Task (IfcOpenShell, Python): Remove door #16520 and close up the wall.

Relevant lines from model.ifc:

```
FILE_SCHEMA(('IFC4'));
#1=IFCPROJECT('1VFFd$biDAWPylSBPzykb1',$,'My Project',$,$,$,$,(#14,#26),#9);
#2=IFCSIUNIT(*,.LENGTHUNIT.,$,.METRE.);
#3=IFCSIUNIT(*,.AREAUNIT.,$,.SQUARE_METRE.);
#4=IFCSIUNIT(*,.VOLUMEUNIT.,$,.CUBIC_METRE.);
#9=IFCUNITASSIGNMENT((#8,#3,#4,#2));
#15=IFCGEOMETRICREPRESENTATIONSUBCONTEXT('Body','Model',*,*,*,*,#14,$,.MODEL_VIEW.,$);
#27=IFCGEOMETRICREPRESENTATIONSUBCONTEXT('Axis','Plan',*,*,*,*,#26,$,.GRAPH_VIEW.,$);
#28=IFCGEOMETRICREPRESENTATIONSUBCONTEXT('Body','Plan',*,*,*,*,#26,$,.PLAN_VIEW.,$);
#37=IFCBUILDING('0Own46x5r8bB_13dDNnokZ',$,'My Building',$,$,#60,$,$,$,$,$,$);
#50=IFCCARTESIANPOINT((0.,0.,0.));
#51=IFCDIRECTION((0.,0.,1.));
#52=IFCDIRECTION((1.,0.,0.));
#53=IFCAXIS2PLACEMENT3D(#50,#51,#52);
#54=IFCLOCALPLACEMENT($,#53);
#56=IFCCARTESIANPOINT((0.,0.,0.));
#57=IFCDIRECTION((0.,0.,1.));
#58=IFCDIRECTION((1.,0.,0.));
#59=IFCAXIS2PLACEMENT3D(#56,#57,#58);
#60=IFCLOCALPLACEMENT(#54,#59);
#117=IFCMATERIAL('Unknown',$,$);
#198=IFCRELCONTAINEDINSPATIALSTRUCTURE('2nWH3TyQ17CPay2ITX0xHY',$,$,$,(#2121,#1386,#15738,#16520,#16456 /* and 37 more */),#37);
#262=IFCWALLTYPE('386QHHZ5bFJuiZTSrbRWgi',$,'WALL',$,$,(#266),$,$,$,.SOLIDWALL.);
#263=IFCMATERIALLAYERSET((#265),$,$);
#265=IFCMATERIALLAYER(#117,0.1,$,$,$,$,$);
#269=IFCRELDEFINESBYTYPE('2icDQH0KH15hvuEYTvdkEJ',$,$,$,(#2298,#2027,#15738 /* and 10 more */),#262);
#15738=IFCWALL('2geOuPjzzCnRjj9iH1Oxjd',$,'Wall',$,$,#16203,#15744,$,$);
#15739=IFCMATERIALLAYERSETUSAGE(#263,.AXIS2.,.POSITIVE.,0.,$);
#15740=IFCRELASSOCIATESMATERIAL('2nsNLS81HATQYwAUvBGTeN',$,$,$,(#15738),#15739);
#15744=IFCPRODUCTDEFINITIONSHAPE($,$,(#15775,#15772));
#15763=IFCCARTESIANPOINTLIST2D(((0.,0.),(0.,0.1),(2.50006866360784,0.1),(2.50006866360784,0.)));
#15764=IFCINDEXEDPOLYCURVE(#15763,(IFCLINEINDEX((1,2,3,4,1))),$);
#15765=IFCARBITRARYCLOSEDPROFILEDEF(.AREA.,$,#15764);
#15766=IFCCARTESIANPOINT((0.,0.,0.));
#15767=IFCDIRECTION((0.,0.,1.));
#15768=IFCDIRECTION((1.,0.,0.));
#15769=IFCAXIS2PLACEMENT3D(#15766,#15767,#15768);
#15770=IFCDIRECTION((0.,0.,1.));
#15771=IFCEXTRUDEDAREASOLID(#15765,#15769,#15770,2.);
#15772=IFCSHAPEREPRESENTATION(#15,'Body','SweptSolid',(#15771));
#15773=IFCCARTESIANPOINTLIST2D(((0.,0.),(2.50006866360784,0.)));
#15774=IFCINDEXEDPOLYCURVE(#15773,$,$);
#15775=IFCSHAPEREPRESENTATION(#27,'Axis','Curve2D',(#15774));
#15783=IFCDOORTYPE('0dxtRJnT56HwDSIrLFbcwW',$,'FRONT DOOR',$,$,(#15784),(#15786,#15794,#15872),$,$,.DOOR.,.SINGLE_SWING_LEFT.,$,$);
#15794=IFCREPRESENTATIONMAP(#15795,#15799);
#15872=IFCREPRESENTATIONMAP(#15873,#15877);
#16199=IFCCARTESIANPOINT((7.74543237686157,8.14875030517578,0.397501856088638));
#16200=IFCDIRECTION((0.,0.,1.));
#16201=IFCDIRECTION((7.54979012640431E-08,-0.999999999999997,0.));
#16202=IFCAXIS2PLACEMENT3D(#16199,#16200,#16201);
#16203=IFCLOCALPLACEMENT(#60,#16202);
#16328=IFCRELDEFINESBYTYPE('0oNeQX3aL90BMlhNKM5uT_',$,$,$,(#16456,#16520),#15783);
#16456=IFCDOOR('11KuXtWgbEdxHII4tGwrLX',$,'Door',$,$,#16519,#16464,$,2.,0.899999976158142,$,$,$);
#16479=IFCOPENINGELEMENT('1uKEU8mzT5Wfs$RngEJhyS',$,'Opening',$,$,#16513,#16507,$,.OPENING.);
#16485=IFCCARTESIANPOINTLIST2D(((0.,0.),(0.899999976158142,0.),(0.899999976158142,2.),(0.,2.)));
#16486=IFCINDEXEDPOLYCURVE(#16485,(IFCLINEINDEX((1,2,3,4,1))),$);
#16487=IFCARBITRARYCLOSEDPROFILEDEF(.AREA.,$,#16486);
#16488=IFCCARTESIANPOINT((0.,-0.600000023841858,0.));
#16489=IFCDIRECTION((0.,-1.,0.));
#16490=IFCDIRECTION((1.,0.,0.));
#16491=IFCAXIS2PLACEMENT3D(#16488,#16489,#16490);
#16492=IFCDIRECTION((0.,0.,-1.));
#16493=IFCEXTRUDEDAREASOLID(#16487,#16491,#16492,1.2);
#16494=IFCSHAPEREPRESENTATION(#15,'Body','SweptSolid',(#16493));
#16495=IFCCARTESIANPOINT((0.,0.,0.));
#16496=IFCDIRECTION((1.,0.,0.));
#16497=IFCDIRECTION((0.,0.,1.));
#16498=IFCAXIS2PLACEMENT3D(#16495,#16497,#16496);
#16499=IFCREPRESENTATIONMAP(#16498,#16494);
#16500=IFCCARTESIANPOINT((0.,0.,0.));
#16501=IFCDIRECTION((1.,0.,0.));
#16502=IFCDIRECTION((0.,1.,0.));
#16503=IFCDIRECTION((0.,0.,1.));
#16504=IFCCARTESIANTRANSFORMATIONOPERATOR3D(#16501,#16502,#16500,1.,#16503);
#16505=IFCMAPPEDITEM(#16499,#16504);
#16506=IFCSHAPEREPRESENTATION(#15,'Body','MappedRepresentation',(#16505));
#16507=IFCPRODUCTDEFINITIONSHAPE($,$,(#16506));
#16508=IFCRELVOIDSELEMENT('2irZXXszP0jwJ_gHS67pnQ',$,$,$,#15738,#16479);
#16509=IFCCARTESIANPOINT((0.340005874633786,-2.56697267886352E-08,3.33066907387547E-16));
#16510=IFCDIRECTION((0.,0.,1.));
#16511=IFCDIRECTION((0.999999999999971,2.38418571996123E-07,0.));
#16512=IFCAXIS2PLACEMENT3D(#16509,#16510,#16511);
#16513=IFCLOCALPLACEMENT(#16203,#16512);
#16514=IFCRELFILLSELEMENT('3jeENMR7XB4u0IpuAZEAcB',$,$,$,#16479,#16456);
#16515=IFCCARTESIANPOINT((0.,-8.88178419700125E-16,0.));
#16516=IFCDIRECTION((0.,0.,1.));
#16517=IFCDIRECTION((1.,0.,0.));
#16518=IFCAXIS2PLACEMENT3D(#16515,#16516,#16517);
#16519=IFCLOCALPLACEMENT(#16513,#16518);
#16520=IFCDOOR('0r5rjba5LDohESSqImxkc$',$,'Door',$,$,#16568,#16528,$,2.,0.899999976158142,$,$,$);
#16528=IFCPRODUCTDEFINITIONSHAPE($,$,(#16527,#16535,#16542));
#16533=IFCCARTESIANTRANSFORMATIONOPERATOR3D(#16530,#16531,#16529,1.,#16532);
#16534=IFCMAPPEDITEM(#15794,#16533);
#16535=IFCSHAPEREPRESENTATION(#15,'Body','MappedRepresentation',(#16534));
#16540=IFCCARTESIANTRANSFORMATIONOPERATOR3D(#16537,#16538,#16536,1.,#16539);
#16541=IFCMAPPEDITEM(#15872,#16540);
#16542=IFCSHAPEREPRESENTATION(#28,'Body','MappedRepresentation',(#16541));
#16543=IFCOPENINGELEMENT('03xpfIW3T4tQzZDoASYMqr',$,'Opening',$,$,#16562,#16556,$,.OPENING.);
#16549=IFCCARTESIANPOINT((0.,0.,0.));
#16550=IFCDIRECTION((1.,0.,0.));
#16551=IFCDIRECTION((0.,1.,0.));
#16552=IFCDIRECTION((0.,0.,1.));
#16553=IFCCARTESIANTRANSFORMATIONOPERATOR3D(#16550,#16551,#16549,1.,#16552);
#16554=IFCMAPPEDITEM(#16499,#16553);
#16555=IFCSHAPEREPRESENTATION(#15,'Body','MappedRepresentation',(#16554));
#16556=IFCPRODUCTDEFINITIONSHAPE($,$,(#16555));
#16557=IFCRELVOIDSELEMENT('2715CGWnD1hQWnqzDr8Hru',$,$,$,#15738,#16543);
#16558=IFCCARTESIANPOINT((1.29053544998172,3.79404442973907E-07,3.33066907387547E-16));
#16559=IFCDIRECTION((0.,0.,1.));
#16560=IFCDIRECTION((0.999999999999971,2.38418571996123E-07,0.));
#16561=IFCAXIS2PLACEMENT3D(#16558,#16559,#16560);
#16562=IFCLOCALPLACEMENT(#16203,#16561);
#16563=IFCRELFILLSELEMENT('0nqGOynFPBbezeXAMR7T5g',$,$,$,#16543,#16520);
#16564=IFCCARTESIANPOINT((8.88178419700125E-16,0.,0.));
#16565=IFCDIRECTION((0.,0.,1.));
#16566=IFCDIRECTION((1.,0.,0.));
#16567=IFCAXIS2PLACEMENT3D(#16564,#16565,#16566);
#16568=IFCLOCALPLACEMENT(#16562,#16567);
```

```python
import ifcopenshell
import ifcopenshell.api.feature
import ifcopenshell.api.root
import ifcopenshell.geom
import ifcopenshell.util.shape

model = ifcopenshell.open("model.ifc")
settings = ifcopenshell.geom.settings()


def volume(element):
    """Net volume in cubic metres, openings subtracted."""
    shape = ifcopenshell.geom.create_shape(settings, element)
    return ifcopenshell.util.shape.get_volume(shape.geometry)


door = model.by_guid("0r5rjba5LDohESSqImxkc$")
opening = door.FillsVoids[0].RelatingOpeningElement
wall = opening.VoidsElements[0].RelatingBuildingElement
before = volume(wall)

ifcopenshell.api.root.remove_product(model, product=door)
ifcopenshell.api.feature.remove_feature(model, feature=opening)

after = volume(wall)

print(f"wall volume {before:.3f} -> {after:.3f} m3")

model.write("model-out.ifc")
```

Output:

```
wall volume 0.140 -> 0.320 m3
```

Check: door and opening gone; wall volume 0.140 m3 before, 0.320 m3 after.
